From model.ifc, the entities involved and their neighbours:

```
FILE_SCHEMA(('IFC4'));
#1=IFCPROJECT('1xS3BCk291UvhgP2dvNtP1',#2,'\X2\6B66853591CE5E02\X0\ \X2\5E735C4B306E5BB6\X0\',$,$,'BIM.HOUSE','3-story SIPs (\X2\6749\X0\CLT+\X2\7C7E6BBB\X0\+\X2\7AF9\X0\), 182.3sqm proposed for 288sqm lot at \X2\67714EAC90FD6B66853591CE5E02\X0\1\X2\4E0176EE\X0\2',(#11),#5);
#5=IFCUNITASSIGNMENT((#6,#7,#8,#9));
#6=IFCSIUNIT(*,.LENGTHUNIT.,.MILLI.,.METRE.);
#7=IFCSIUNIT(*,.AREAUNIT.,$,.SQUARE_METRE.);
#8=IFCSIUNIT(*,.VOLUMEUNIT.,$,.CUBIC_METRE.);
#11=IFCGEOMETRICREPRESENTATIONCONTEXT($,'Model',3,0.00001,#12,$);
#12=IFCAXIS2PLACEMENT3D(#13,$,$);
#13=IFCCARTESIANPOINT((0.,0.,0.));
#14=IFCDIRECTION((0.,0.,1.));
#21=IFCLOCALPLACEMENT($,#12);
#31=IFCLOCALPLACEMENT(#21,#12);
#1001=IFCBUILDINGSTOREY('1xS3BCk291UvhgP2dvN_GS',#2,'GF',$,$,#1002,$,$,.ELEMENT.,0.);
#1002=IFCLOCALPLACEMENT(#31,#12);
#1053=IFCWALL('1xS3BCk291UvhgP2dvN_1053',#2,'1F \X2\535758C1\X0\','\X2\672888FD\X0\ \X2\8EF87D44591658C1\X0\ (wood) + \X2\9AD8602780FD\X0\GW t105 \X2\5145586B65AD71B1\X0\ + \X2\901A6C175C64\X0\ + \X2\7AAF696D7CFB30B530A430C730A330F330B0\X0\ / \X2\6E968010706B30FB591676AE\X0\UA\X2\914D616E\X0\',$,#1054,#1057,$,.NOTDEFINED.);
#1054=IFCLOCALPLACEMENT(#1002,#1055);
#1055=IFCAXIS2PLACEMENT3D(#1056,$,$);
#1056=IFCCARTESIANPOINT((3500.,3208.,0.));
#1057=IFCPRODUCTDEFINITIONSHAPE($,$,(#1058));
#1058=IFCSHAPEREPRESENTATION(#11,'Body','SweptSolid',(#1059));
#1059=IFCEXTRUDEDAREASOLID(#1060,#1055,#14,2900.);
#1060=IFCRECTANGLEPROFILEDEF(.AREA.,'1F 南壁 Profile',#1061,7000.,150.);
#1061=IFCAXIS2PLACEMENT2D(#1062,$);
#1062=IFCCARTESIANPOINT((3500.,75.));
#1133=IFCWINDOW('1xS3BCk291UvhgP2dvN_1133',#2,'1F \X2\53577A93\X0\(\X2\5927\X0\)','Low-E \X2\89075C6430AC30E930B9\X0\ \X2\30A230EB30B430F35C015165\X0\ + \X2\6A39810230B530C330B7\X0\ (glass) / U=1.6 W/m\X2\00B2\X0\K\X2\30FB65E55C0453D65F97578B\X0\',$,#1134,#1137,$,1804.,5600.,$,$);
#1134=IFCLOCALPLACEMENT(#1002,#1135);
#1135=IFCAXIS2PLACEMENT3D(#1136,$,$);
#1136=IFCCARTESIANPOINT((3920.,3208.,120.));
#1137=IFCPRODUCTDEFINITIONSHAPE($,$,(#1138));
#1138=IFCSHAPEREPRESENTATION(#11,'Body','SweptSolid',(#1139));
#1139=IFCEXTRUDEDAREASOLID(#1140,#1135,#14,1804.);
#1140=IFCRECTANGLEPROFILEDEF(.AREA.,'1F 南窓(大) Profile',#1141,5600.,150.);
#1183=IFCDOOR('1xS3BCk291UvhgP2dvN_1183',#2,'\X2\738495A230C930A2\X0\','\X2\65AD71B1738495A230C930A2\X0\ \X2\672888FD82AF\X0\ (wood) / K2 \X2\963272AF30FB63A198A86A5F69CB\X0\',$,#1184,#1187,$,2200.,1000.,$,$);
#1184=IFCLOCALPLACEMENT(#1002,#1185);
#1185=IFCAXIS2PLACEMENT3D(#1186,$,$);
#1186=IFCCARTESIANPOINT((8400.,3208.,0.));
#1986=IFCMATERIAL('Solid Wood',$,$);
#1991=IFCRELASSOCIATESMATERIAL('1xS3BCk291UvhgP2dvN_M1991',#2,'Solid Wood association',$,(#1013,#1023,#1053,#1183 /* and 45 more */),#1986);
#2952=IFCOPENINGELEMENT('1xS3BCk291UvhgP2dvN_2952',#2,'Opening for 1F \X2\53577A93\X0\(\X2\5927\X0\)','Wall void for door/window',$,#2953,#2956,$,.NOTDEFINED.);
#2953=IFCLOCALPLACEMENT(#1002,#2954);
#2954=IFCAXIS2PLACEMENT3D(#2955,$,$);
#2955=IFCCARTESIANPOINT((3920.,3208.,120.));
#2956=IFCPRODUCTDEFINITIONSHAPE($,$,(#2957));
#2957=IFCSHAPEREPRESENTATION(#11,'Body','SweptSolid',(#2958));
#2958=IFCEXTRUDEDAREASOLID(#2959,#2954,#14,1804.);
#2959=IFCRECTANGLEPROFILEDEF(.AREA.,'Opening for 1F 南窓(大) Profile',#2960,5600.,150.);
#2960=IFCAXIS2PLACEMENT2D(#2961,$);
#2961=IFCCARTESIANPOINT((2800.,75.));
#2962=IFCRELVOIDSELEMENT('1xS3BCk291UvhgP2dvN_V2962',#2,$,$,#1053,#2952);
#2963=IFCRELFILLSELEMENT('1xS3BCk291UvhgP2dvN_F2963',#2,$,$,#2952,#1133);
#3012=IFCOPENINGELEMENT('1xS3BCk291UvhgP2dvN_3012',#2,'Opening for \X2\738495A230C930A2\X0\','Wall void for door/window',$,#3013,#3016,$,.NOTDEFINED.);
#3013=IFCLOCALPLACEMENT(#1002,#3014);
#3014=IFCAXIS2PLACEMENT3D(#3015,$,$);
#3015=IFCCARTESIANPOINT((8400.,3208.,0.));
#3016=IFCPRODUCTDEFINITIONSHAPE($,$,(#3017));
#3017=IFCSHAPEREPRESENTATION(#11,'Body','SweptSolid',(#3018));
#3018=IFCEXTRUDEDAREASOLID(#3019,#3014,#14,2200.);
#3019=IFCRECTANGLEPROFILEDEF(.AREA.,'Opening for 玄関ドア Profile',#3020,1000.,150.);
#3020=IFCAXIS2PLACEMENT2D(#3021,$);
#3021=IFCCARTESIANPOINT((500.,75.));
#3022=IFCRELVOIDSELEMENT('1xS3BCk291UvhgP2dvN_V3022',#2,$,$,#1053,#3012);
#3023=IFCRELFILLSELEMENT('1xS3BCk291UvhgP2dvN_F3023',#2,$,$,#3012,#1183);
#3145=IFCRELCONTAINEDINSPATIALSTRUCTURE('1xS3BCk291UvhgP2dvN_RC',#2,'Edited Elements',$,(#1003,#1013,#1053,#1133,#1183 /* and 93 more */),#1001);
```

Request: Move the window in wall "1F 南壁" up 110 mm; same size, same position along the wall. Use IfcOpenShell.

```python
import numpy as np
import ifcopenshell
import ifcopenshell.api.geometry
import ifcopenshell.util.placement
import ifcopenshell.util.unit

model = ifcopenshell.open("model.ifc")
unit_scale = ifcopenshell.util.unit.calculate_unit_scale(model)

window = model.by_id(1133)
opening = window.FillsVoids[0].RelatingOpeningElement
dz = 0.11 / unit_scale

shift = np.array([0.0, 0.0, dz])
# The window is not placed relative to its opening, so move both.
for product in (opening, window):
    matrix = ifcopenshell.util.placement.get_local_placement(product.ObjectPlacement)
    matrix[:3, 3] += shift
    ifcopenshell.api.geometry.edit_object_placement(model, product=product, matrix=matrix, is_si=False)

print(f"moved by {dz * unit_scale:+.3f} m")

model.write("model_v2.ifc")
```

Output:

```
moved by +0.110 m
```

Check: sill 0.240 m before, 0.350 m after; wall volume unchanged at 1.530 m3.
